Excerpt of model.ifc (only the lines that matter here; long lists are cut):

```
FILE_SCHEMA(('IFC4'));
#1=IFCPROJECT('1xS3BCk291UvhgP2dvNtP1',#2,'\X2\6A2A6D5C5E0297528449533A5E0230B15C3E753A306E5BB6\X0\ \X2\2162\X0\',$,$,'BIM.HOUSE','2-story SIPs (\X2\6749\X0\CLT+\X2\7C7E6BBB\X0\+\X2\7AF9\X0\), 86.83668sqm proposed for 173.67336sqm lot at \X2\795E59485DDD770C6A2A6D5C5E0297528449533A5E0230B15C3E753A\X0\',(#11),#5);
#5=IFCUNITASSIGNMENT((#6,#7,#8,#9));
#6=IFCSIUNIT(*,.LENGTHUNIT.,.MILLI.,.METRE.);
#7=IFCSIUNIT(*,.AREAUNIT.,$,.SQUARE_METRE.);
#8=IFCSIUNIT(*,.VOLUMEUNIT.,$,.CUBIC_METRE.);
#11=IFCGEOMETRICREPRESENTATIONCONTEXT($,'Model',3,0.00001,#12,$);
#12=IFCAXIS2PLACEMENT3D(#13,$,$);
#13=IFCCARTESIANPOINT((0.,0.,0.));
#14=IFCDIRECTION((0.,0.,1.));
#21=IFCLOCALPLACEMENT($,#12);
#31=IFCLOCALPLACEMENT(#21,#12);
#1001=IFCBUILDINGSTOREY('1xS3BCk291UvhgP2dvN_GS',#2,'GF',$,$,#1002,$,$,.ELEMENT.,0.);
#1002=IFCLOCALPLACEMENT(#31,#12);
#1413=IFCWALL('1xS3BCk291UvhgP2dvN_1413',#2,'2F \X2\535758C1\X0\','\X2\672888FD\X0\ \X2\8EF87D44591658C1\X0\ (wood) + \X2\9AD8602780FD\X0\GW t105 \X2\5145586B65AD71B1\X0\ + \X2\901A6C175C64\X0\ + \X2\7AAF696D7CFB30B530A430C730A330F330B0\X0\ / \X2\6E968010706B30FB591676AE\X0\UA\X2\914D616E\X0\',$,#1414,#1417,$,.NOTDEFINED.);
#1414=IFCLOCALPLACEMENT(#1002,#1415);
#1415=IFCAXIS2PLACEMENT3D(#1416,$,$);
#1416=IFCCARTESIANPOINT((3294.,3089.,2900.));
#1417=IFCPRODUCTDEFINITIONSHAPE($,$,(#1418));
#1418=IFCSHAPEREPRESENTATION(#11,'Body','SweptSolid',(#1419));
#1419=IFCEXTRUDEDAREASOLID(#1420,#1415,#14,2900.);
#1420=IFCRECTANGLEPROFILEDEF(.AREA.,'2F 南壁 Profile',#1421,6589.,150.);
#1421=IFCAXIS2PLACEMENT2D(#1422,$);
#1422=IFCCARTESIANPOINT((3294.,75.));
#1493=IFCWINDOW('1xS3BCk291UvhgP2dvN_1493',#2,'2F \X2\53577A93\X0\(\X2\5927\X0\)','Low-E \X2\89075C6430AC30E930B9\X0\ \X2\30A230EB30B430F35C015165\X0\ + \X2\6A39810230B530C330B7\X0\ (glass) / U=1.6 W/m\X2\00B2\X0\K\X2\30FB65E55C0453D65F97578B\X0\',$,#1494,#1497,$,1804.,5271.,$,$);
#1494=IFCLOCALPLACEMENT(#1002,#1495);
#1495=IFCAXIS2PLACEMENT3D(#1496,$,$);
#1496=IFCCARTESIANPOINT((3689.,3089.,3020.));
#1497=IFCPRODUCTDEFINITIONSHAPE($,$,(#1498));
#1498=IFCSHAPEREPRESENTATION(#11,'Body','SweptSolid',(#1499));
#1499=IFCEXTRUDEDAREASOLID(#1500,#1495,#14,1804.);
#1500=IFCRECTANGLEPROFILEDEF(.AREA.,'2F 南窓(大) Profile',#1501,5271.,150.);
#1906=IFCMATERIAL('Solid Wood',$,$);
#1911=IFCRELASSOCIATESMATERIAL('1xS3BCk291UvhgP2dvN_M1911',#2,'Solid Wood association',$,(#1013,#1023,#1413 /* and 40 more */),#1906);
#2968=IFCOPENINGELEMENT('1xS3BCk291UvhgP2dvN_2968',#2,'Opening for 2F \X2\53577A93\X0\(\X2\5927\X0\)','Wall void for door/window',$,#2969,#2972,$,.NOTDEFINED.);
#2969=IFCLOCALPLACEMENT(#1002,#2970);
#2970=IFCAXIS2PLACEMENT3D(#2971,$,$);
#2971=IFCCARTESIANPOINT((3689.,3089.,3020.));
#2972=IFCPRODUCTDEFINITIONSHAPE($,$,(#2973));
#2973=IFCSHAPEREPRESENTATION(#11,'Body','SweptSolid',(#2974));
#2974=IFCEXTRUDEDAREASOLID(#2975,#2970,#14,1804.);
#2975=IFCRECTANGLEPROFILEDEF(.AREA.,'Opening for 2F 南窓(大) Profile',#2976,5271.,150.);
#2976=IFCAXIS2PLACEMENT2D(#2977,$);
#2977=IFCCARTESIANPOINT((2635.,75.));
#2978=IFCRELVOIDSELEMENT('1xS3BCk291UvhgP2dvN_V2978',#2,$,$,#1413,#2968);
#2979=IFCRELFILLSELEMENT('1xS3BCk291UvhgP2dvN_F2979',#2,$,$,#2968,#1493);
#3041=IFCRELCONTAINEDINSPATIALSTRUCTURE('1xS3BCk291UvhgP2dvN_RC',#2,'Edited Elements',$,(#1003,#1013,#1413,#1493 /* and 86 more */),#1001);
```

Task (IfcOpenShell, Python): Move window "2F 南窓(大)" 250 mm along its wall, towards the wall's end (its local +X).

```python
import ifcopenshell
import ifcopenshell.api.geometry
import ifcopenshell.util.placement

model = ifcopenshell.open("model.ifc")

window = model.by_id(1493)
opening = window.FillsVoids[0].RelatingOpeningElement
wall = opening.VoidsElements[0].RelatingBuildingElement

wall_matrix = ifcopenshell.util.placement.get_local_placement(wall.ObjectPlacement)
shift = wall_matrix[:3, 0] * 250.0
before = ifcopenshell.util.placement.get_local_placement(window.ObjectPlacement)[:3, 3].copy()

# The window is not placed relative to its opening, so move both.
for product in (opening, window):
    matrix = ifcopenshell.util.placement.get_local_placement(product.ObjectPlacement)
    matrix[:3, 3] += shift
    ifcopenshell.api.geometry.edit_object_placement(model, product=product, matrix=matrix, is_si=False)

after = ifcopenshell.util.placement.get_local_placement(window.ObjectPlacement)[:3, 3]
print("window moved by", (after - before).round(3) + 0.0)

model.write("model_updated.ifc")
```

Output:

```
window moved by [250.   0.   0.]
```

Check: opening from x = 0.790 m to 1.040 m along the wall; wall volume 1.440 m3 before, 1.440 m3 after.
